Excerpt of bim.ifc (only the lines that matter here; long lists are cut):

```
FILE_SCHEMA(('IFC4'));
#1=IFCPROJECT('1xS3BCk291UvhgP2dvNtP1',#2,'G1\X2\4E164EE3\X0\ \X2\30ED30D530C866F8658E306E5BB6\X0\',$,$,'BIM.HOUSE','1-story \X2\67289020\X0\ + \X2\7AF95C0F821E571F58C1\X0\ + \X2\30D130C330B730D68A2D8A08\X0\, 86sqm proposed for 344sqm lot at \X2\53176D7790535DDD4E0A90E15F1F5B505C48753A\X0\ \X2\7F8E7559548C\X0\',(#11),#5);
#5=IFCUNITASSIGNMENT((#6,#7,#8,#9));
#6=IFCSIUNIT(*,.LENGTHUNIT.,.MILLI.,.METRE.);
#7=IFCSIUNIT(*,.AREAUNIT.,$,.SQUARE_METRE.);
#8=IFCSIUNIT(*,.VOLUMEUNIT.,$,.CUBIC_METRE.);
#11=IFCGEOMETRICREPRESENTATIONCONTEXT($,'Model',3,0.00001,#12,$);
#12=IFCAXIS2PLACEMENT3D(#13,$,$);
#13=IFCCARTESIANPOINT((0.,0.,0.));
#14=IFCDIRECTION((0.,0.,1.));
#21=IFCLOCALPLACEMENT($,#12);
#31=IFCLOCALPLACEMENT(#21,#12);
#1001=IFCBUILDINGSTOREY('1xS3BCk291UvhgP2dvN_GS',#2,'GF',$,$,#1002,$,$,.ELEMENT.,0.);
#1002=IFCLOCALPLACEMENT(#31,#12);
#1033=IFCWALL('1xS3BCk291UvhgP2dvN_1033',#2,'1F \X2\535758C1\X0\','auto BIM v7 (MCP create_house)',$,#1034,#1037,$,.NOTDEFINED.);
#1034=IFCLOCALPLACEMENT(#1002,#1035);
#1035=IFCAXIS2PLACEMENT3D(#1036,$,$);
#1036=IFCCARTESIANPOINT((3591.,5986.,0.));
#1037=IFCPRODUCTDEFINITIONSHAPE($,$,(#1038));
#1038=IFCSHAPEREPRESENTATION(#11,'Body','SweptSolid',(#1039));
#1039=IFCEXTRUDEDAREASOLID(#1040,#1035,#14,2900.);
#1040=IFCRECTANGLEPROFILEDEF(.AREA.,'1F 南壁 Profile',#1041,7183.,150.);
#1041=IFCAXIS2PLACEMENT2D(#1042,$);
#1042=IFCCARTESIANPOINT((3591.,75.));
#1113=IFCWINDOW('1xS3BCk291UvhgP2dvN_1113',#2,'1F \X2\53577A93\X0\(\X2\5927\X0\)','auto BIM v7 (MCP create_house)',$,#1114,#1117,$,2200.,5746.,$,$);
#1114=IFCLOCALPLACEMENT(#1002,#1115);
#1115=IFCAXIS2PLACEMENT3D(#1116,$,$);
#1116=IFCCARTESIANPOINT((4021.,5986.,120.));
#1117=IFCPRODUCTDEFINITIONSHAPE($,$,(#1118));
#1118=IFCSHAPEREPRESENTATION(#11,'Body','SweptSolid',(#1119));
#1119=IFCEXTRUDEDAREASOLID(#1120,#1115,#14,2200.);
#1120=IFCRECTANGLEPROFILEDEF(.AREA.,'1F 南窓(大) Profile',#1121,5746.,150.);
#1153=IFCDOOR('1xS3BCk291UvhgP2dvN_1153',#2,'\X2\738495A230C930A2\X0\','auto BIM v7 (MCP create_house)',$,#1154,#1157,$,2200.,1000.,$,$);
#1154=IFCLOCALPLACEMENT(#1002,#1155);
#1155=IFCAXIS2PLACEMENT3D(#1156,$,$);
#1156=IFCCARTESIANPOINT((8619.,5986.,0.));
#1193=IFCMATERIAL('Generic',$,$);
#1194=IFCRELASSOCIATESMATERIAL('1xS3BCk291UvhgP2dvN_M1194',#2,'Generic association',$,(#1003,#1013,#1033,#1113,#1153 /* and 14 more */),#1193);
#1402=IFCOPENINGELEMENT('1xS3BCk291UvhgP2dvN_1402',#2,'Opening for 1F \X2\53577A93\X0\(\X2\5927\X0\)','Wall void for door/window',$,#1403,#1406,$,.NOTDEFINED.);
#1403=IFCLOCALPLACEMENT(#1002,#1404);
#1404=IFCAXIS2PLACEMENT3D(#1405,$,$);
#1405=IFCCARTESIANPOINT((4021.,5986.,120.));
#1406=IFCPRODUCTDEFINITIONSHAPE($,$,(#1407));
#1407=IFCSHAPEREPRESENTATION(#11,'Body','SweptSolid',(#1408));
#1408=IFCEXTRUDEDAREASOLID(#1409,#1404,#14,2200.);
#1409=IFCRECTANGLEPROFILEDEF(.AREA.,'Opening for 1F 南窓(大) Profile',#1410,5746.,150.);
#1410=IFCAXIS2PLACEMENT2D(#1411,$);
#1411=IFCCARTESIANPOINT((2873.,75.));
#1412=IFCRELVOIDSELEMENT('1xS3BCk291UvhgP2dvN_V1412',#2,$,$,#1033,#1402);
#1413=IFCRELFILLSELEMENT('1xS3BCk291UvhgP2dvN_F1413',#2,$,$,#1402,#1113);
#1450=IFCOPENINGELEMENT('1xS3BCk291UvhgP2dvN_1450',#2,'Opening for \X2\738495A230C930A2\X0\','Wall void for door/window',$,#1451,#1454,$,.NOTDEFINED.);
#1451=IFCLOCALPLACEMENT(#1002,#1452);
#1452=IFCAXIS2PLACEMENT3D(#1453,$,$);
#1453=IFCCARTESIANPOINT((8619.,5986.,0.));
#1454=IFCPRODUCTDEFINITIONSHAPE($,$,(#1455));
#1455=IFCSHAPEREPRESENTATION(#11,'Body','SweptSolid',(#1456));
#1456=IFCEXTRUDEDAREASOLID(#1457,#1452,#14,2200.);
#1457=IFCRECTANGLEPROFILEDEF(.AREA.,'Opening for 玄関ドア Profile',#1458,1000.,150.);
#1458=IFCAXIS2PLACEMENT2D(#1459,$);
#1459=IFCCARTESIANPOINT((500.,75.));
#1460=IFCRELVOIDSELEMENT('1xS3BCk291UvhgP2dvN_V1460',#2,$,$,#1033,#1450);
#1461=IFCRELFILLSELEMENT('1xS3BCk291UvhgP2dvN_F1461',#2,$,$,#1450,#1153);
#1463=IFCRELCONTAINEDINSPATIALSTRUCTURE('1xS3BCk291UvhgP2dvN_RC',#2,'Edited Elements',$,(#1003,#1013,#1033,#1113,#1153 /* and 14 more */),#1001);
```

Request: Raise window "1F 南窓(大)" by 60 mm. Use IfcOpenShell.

```python
import numpy as np
import ifcopenshell
import ifcopenshell.api.geometry
import ifcopenshell.util.placement
import ifcopenshell.util.unit

model = ifcopenshell.open("bim.ifc")
unit_scale = ifcopenshell.util.unit.calculate_unit_scale(model)

window = model.by_id(1113)
opening = window.FillsVoids[0].RelatingOpeningElement
dz = 0.06 / unit_scale

shift = np.array([0.0, 0.0, dz])
# The window is not placed relative to its opening, so move both.
for product in (opening, window):
    matrix = ifcopenshell.util.placement.get_local_placement(product.ObjectPlacement)
    matrix[:3, 3] += shift
    ifcopenshell.api.geometry.edit_object_placement(model, product=product, matrix=matrix, is_si=False)

print(f"moved by {dz * unit_scale:+.3f} m")

model.write("bim_v2.ifc")
```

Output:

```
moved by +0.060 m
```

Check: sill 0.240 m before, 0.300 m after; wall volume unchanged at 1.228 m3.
